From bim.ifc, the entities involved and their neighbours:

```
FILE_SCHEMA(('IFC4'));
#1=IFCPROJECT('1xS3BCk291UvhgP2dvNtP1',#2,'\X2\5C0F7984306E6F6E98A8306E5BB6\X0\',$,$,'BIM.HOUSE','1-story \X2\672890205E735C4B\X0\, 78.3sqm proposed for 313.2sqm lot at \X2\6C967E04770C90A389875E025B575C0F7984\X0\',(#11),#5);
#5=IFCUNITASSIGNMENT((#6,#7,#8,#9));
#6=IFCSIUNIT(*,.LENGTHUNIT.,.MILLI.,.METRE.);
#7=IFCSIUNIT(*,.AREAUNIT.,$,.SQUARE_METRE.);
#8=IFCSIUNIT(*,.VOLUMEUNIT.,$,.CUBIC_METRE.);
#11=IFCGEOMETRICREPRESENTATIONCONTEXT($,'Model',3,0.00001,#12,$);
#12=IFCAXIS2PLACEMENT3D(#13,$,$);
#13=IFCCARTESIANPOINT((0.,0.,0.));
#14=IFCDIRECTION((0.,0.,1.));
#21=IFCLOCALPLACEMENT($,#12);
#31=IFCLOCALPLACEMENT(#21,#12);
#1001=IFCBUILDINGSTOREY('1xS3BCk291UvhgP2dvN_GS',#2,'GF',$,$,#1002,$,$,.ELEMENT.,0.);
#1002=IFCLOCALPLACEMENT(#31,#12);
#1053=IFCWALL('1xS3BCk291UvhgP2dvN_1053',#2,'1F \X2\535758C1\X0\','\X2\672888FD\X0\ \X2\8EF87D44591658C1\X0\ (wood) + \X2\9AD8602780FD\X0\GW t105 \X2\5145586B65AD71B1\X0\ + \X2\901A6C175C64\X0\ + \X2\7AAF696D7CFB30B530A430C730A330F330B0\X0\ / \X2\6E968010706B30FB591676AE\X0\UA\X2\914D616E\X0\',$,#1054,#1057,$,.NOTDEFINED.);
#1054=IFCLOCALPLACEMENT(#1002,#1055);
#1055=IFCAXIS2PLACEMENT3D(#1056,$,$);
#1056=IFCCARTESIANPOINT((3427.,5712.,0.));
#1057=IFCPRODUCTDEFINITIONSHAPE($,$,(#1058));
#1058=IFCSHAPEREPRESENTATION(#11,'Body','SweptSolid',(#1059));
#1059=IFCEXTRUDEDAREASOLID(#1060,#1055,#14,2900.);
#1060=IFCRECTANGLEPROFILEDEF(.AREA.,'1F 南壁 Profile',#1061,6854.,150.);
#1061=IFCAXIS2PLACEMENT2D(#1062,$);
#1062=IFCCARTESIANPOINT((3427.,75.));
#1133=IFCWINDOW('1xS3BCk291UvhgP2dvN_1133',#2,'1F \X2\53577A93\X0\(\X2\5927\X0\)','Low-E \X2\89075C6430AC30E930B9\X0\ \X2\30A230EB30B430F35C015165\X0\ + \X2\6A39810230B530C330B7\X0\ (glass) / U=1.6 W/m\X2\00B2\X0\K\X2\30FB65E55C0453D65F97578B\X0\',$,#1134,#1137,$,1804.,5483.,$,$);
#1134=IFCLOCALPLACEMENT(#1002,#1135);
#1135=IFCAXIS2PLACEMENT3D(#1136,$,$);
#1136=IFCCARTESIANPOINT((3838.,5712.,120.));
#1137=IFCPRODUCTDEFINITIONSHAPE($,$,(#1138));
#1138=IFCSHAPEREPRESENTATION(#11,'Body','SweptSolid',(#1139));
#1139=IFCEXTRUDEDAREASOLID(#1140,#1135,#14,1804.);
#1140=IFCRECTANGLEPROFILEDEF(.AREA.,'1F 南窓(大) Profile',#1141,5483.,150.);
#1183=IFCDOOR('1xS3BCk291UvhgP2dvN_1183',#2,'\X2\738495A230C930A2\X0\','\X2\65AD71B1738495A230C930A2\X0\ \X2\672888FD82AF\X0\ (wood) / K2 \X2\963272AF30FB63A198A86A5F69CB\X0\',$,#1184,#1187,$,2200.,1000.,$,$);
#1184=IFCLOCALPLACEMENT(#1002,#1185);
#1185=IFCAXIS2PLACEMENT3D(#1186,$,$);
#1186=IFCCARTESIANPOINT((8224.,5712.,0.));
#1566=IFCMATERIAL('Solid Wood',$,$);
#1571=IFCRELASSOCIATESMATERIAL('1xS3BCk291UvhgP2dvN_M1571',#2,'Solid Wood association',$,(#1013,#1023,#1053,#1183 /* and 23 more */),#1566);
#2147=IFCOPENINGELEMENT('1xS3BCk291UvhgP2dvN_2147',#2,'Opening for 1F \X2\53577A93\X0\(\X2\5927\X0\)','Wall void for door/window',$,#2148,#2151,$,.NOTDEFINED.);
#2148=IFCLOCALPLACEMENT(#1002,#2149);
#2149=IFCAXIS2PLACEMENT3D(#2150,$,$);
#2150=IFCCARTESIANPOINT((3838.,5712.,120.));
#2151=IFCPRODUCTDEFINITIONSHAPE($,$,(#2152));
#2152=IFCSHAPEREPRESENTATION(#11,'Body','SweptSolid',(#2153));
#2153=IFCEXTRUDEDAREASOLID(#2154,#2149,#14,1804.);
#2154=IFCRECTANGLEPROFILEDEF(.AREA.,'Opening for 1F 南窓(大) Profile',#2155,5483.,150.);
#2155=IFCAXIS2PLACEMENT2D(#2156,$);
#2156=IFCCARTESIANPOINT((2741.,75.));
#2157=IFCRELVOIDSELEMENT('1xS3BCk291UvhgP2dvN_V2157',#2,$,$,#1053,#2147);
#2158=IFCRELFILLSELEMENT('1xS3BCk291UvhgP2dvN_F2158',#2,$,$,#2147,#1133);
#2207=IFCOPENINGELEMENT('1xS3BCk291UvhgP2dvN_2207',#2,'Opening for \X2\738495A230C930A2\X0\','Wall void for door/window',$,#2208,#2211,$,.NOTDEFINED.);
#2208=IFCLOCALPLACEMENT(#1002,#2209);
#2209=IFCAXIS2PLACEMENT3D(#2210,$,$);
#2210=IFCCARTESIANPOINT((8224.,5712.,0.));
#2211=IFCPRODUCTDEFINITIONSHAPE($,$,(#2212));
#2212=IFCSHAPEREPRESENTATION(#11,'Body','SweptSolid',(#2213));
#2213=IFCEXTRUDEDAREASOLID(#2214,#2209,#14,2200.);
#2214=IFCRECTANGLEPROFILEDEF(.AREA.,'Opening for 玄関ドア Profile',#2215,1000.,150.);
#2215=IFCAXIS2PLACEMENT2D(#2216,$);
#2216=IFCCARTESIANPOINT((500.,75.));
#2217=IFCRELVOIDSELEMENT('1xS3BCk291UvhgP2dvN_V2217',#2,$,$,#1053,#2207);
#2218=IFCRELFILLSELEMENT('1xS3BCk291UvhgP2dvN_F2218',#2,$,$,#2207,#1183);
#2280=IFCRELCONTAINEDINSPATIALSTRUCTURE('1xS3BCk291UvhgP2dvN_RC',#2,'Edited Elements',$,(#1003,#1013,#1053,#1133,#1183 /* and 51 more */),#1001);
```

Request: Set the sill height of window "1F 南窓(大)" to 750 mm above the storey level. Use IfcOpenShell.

```python
import numpy as np
import ifcopenshell
import ifcopenshell.api.geometry
import ifcopenshell.geom
import ifcopenshell.util.element
import ifcopenshell.util.placement
import ifcopenshell.util.shape
import ifcopenshell.util.unit

model = ifcopenshell.open("bim.ifc")
unit_scale = ifcopenshell.util.unit.calculate_unit_scale(model)

window = model.by_guid("1xS3BCk291UvhgP2dvN_1133")
opening = window.FillsVoids[0].RelatingOpeningElement
storey = ifcopenshell.util.element.get_container(window, ifc_class="IfcBuildingStorey")
level = ifcopenshell.util.placement.get_local_placement(storey.ObjectPlacement)[2, 3]

# The opening's origin need not be at the sill, so measure its lowest point.
shape = ifcopenshell.geom.create_shape(ifcopenshell.geom.settings(), opening)
bottom = ifcopenshell.util.shape.get_shape_bottom_elevation(shape, shape.geometry) / unit_scale
dz = level + 750.0 - bottom

shift = np.array([0.0, 0.0, dz])
# The window is not placed relative to its opening, so move both.
for product in (opening, window):
    matrix = ifcopenshell.util.placement.get_local_placement(product.ObjectPlacement)
    matrix[:3, 3] += shift
    ifcopenshell.api.geometry.edit_object_placement(model, product=product, matrix=matrix, is_si=False)

print(f"moved by {dz * unit_scale:+.3f} m")

model.write("bim-out.ifc")
```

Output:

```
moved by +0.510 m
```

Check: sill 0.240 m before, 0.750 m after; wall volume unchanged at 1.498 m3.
